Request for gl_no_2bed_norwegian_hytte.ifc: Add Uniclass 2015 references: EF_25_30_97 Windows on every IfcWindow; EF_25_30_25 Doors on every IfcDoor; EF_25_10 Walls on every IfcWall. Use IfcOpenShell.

First a look at what the model holds.

```python
import ifcopenshell

model = ifcopenshell.open("gl_no_2bed_norwegian_hytte.ifc")
print(model.schema)
print("classifications:", [c.Name for c in model.by_type("IfcClassification")])
for ifc_class in ("IfcDoor", "IfcRoof", "IfcStair", "IfcWall", "IfcWindow"):
    print(ifc_class, len(model.by_type(ifc_class)))
```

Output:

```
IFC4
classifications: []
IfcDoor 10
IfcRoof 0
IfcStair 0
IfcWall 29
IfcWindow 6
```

```python
import ifcopenshell
import ifcopenshell.api.classification

model = ifcopenshell.open("gl_no_2bed_norwegian_hytte.ifc")

system = ifcopenshell.api.classification.add_classification(model, classification="Uniclass 2015")

codes = {
    "IfcWindow": ("EF_25_30_97", "Windows"),
    "IfcDoor": ("EF_25_30_25", "Doors"),
    "IfcWall": ("EF_25_10", "Walls"),
}
for ifc_class, (code, name) in codes.items():
    products = model.by_type(ifc_class)
    ifcopenshell.api.classification.add_reference(
        model, products=products, classification=system, identification=code, name=name
    )
    print(code, len(products))

model.write("gl_no_2bed_norwegian_hytte-out.ifc")
```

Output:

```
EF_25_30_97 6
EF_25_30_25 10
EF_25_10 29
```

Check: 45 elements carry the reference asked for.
